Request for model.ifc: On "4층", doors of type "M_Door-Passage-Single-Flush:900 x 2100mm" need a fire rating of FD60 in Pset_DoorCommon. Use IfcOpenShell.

First a look at what the model holds.

```python
import ifcopenshell
import ifcopenshell.util.element

model = ifcopenshell.open("model.ifc")
print(model.schema)
storey = next(s for s in model.by_type("IfcBuildingStorey") if s.Name == "4층")
doors = [e for e in ifcopenshell.util.element.get_decomposition(storey) if e.is_a("IfcDoor")]
seen = {}
for e in doors:
    element_type = ifcopenshell.util.element.get_type(e)
    key = (element_type.Name if element_type != e and element_type else None, ifcopenshell.util.element.get_pset(e, "Pset_DoorCommon", "FireRating"))
    seen[key] = seen.get(key, 0) + 1
for (name, value), count in sorted(seen.items(), key=str):
    print(count, "x", name, "|", value)
```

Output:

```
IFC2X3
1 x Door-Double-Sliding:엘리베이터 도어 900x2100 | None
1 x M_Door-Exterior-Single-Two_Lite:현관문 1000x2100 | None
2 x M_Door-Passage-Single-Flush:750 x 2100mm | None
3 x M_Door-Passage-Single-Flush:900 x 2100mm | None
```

```python
import ifcopenshell
import ifcopenshell.api.pset
import ifcopenshell.util.element

model = ifcopenshell.open("model.ifc")

storey = next(s for s in model.by_type("IfcBuildingStorey") if s.Name == "4층")
doors = [e for e in ifcopenshell.util.element.get_decomposition(storey) if e.is_a("IfcDoor")]

count = 0
for e in doors:
    element_type = ifcopenshell.util.element.get_type(e)
    if element_type in (None, e) or element_type.Name != "M_Door-Passage-Single-Flush:900 x 2100mm":
        continue
    # add_pset returns the element's existing set when there is one.
    pset = ifcopenshell.api.pset.add_pset(model, product=e, name="Pset_DoorCommon")
    ifcopenshell.api.pset.edit_pset(model, pset=pset, properties={"FireRating": "FD60"})
    count += 1

print(count, "doors updated")

model.write("model_updated.ifc")
```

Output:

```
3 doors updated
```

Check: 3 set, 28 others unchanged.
